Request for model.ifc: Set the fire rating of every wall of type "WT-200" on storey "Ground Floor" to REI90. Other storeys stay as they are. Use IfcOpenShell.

First a look at what the model holds.

```python
import ifcopenshell
import ifcopenshell.util.element

model = ifcopenshell.open("model.ifc")
print(model.schema)
storey = next(s for s in model.by_type("IfcBuildingStorey") if s.Name == "Ground Floor")
walls = [e for e in ifcopenshell.util.element.get_decomposition(storey) if e.is_a("IfcWall")]
seen = {}
for e in walls:
    element_type = ifcopenshell.util.element.get_type(e)
    key = (element_type.Name if element_type != e and element_type else None, ifcopenshell.util.element.get_pset(e, "Pset_WallCommon", "FireRating"))
    seen[key] = seen.get(key, 0) + 1
for (name, value), count in sorted(seen.items(), key=str):
    print(count, "x", name, "|", value)
```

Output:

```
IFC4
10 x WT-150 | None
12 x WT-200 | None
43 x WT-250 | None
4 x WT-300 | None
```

```python
import ifcopenshell
import ifcopenshell.api.pset
import ifcopenshell.util.element

model = ifcopenshell.open("model.ifc")

storey = next(s for s in model.by_type("IfcBuildingStorey") if s.Name == "Ground Floor")
walls = [e for e in ifcopenshell.util.element.get_decomposition(storey) if e.is_a("IfcWall")]

count = 0
for e in walls:
    element_type = ifcopenshell.util.element.get_type(e)
    if element_type in (None, e) or element_type.Name != "WT-200":
        continue
    # add_pset returns the element's existing set when there is one.
    pset = ifcopenshell.api.pset.add_pset(model, product=e, name="Pset_WallCommon")
    ifcopenshell.api.pset.edit_pset(model, pset=pset, properties={"FireRating": "REI90"})
    count += 1

print(count, "walls updated")

model.write("model-out.ifc")
```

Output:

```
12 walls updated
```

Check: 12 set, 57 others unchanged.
